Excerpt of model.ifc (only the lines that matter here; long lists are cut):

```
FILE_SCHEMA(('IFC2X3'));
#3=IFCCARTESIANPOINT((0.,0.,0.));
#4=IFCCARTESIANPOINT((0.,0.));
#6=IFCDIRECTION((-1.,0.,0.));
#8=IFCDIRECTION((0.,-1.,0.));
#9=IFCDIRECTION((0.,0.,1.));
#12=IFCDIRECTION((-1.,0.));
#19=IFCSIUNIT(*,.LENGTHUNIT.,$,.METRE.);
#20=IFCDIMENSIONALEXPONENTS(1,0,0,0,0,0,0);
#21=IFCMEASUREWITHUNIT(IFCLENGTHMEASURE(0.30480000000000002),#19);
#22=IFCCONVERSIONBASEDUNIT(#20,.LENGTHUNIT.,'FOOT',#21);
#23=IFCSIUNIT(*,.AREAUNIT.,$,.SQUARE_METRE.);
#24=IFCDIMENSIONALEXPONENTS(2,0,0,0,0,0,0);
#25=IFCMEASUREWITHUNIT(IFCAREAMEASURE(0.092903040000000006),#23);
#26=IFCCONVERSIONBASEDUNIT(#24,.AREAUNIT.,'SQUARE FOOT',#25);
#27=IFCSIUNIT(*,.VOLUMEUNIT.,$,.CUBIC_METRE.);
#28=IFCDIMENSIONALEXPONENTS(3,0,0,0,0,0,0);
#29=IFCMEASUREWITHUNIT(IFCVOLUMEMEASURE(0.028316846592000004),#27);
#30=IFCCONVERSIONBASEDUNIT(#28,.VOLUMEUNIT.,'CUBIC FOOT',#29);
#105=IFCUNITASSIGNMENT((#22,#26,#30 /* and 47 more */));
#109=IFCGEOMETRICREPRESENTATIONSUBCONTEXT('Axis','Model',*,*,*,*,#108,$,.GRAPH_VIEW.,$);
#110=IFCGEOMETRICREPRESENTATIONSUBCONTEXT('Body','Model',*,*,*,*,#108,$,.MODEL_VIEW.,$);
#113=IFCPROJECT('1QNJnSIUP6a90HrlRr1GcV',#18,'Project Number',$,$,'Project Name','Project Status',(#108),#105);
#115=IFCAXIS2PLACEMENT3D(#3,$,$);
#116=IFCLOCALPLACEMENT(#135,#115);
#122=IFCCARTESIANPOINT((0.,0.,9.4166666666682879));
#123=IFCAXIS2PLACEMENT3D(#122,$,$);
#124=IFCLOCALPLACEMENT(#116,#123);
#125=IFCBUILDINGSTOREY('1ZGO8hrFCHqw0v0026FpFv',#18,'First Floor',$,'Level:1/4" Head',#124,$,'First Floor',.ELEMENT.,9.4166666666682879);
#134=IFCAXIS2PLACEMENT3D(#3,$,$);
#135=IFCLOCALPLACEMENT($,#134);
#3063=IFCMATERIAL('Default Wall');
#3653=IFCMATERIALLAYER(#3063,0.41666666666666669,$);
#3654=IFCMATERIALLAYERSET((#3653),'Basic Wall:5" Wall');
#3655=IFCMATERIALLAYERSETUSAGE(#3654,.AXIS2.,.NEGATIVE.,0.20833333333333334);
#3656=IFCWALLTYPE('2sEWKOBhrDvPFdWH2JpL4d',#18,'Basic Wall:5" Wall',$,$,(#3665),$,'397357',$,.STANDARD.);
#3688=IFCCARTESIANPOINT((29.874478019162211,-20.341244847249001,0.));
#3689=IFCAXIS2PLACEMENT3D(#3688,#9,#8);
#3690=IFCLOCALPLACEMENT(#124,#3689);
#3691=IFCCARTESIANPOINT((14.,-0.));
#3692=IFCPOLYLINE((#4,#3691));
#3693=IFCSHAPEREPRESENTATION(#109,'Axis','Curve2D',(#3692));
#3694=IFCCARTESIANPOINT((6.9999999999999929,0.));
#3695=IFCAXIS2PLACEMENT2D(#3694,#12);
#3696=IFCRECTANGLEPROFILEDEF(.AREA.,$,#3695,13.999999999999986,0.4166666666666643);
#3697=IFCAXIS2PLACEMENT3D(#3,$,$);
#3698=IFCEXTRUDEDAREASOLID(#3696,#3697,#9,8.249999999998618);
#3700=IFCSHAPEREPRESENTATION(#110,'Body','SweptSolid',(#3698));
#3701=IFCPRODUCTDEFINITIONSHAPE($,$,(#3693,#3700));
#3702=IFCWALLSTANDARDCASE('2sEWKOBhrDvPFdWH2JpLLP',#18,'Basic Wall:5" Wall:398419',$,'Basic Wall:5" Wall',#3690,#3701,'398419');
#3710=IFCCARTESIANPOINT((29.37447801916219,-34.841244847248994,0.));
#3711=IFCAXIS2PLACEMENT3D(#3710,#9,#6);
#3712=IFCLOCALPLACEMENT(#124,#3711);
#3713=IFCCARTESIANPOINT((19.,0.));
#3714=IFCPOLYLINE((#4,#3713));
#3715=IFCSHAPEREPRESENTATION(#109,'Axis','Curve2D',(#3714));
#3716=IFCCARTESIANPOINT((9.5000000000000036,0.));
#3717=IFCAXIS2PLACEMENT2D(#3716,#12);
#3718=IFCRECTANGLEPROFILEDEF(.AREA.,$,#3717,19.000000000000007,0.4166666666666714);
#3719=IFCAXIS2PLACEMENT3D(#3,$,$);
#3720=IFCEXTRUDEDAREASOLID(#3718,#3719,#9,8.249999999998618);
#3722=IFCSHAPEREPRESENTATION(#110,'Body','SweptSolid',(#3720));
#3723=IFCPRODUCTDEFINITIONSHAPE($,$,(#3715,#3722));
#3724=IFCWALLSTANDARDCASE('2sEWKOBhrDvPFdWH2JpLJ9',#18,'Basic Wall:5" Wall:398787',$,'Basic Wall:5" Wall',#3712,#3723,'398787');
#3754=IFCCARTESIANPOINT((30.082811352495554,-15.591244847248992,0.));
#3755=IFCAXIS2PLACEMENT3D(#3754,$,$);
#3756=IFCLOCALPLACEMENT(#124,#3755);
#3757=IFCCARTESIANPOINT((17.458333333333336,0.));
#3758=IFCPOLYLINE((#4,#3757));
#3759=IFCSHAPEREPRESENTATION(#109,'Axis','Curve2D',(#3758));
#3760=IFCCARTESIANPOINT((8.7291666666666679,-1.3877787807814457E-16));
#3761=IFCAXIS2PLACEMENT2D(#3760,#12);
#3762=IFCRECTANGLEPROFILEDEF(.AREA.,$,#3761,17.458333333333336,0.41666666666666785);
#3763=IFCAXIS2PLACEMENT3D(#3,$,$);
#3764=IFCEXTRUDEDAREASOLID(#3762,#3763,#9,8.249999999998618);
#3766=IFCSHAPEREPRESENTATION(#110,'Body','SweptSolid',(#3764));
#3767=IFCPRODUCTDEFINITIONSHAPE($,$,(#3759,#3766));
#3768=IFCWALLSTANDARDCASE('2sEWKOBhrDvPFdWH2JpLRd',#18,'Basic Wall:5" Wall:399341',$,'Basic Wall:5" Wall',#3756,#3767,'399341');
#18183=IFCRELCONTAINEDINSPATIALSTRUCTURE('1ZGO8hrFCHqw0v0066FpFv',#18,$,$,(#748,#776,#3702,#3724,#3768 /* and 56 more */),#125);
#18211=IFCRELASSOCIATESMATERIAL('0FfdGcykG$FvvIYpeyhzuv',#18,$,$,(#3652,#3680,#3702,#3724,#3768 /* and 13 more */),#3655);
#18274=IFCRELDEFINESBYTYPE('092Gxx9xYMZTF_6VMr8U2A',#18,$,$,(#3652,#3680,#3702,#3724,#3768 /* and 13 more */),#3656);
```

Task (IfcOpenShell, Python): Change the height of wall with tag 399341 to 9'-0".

```python
import ifcopenshell
import ifcopenshell.geom
import ifcopenshell.util.representation
import ifcopenshell.util.shape
import ifcopenshell.util.unit

model = ifcopenshell.open("model.ifc")
unit_scale = ifcopenshell.util.unit.calculate_unit_scale(model)
settings = ifcopenshell.geom.settings()


def volume(element):
    """Net volume in cubic metres, openings subtracted."""
    shape = ifcopenshell.geom.create_shape(settings, element)
    return ifcopenshell.util.shape.get_volume(shape.geometry)


wall = model.by_guid("2sEWKOBhrDvPFdWH2JpLRd")
before = volume(wall)

body = ifcopenshell.util.representation.get_representation(wall, "Model", "Body")
solid = body.Items[0]
old_height = solid.Depth
solid.Depth = 108 * 0.0254 / unit_scale
after = volume(wall)

print(f"height {old_height:g} -> {solid.Depth:g}, volume {before:.3f} -> {after:.3f} m3")

model.write("model_v2.ifc")
```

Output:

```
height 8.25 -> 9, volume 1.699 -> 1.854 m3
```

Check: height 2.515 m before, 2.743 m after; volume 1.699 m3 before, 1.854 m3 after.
